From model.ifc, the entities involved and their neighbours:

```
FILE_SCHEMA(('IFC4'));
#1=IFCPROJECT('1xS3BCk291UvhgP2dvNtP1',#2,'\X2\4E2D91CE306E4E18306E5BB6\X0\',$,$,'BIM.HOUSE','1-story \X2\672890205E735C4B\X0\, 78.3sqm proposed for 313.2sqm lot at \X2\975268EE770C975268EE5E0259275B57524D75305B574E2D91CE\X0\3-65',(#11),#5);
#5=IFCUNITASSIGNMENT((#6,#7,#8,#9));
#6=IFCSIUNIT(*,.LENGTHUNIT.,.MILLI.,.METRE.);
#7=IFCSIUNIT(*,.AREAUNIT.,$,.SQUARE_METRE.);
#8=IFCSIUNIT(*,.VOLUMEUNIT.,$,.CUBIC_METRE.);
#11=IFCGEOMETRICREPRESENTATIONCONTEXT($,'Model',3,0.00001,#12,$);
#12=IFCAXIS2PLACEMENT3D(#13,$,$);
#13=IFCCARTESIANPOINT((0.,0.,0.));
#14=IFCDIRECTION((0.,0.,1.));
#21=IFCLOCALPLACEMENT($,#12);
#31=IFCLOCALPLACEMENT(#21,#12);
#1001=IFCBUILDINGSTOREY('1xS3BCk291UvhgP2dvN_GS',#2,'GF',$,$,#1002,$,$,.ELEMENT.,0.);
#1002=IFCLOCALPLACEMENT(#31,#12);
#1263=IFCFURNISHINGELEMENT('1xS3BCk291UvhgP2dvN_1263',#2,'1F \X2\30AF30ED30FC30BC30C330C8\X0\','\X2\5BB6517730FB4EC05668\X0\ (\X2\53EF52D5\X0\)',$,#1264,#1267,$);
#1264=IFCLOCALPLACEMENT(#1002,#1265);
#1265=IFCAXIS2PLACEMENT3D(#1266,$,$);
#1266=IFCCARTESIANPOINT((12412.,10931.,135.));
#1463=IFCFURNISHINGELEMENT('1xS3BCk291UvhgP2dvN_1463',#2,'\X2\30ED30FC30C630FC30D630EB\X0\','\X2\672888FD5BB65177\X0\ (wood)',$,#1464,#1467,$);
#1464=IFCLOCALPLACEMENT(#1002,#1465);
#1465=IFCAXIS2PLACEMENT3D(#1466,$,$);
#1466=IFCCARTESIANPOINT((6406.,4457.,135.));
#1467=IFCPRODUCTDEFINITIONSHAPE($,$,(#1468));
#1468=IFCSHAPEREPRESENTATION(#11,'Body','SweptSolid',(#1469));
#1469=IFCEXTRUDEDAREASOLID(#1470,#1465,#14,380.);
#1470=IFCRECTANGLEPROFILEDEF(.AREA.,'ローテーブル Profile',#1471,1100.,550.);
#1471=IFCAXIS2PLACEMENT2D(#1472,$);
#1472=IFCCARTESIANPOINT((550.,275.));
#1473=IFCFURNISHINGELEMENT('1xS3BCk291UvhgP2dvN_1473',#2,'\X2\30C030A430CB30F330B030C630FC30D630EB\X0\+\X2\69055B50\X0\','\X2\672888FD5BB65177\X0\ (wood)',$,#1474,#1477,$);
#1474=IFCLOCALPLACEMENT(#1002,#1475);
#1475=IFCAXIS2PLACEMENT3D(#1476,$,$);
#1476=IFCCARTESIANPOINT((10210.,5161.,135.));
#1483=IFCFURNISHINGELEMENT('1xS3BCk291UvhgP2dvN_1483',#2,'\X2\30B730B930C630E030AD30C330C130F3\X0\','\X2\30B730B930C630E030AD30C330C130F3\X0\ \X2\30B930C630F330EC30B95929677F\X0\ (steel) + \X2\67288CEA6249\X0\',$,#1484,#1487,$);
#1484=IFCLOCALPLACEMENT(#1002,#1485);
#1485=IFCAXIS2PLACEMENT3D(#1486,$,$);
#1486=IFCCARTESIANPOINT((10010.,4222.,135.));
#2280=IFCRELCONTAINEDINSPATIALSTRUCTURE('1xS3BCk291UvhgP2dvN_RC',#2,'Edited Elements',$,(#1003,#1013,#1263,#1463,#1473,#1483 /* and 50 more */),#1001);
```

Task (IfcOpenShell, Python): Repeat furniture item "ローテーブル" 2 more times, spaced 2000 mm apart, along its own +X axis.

```python
import ifcopenshell
import ifcopenshell.api.geometry
import ifcopenshell.api.root
import ifcopenshell.util.element
import ifcopenshell.util.placement
import ifcopenshell.util.unit

model = ifcopenshell.open("model.ifc")
unit_scale = ifcopenshell.util.unit.calculate_unit_scale(model)


def reuse_history(source, copy):
    """copy_class also copies each property set's owner history, people and application; keep the originals."""
    for rel in copy.IsDefinedBy:
        if rel.is_a("IfcRelDefinesByProperties") and (history := rel.RelatingPropertyDefinition.OwnerHistory):
            rel.RelatingPropertyDefinition.OwnerHistory = source.OwnerHistory
            ifcopenshell.util.element.remove_deep2(model, history)


source = model.by_id(1463)
base = ifcopenshell.util.placement.get_local_placement(source.ObjectPlacement)
step = base[:3, 0] * 2 / unit_scale

for i in range(1, 3):
    copy = ifcopenshell.api.root.copy_class(model, product=source)
    copy.Representation = ifcopenshell.util.element.copy_deep(
        model, source.Representation, exclude=["IfcGeometricRepresentationContext", "IfcRepresentationMap"]
    )
    reuse_history(source, copy)
    matrix = base.copy()
    matrix[:3, 3] += i * step
    print("added at", matrix[:3, 3].round(3) + 0.0)
    ifcopenshell.api.geometry.edit_object_placement(model, product=copy, matrix=matrix, is_si=False)

model.write("model_v2.ifc")
```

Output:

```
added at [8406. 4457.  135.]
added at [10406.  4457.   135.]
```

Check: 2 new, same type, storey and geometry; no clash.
